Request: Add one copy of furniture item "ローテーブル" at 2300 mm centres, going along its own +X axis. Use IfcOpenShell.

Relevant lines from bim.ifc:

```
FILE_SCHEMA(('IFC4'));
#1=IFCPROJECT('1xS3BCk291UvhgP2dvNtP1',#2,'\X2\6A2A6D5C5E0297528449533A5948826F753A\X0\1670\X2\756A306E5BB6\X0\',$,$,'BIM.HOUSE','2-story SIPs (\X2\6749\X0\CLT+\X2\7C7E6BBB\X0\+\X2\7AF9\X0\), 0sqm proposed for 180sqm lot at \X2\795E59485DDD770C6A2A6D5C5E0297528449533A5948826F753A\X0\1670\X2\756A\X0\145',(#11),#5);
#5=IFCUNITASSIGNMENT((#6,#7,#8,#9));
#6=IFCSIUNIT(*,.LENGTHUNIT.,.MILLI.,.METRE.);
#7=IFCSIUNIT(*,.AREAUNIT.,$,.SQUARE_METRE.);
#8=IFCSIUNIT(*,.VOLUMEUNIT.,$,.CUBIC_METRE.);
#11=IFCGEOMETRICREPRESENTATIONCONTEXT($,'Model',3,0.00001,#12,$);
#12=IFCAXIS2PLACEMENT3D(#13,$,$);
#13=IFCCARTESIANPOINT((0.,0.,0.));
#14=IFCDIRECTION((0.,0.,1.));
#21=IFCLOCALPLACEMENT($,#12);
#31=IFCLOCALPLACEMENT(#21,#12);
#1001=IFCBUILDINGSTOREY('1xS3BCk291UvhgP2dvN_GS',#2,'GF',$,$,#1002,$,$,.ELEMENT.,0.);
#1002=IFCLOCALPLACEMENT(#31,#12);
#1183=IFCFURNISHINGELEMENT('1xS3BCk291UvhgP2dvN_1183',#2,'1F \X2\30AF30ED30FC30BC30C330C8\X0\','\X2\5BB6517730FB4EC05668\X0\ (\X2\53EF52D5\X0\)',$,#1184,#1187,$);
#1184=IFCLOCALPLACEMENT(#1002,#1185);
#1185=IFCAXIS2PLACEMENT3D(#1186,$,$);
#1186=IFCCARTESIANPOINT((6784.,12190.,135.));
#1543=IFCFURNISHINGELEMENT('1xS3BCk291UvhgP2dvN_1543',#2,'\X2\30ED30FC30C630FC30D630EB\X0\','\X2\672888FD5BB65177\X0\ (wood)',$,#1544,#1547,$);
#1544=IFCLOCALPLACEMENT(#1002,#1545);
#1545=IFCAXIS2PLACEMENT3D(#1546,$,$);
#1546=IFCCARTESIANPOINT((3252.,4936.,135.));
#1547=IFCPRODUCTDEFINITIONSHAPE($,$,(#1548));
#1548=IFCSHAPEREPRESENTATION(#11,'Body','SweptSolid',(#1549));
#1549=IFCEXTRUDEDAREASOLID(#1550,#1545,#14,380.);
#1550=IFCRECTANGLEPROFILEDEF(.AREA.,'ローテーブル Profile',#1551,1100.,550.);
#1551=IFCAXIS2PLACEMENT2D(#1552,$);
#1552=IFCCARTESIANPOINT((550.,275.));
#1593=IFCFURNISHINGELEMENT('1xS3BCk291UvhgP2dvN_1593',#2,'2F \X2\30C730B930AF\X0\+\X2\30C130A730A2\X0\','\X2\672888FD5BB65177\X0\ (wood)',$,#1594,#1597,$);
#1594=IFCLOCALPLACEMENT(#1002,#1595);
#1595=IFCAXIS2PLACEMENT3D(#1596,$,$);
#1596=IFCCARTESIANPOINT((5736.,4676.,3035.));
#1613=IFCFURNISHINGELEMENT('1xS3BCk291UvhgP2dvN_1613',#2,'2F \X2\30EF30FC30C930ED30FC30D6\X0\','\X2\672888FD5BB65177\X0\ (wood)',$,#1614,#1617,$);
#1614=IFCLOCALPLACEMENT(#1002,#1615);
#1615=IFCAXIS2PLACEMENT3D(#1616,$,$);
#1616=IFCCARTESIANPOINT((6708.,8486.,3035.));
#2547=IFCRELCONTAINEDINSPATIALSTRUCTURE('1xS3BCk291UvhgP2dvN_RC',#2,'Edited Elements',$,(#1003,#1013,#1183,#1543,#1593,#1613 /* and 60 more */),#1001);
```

```python
import ifcopenshell
import ifcopenshell.api.geometry
import ifcopenshell.api.root
import ifcopenshell.util.element
import ifcopenshell.util.placement
import ifcopenshell.util.unit

model = ifcopenshell.open("bim.ifc")
unit_scale = ifcopenshell.util.unit.calculate_unit_scale(model)


def reuse_history(source, copy):
    """copy_class also copies each property set's owner history, people and application; keep the originals."""
    for rel in copy.IsDefinedBy:
        if rel.is_a("IfcRelDefinesByProperties") and (history := rel.RelatingPropertyDefinition.OwnerHistory):
            rel.RelatingPropertyDefinition.OwnerHistory = source.OwnerHistory
            ifcopenshell.util.element.remove_deep2(model, history)


source = model.by_guid("1xS3BCk291UvhgP2dvN_1543")
base = ifcopenshell.util.placement.get_local_placement(source.ObjectPlacement)
step = base[:3, 0] * 2.3 / unit_scale

for i in range(1, 2):
    copy = ifcopenshell.api.root.copy_class(model, product=source)
    copy.Representation = ifcopenshell.util.element.copy_deep(
        model, source.Representation, exclude=["IfcGeometricRepresentationContext", "IfcRepresentationMap"]
    )
    reuse_history(source, copy)
    matrix = base.copy()
    matrix[:3, 3] += i * step
    print("added at", matrix[:3, 3].round(3) + 0.0)
    ifcopenshell.api.geometry.edit_object_placement(model, product=copy, matrix=matrix, is_si=False)

model.write("bim_edited.ifc")
```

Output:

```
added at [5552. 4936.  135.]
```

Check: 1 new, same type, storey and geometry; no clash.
